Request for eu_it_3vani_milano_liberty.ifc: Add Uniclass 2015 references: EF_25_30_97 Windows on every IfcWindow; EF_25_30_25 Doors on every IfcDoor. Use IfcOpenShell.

First a look at what the model holds.

```python
import ifcopenshell

model = ifcopenshell.open("eu_it_3vani_milano_liberty.ifc")
print(model.schema)
print("classifications:", [c.Name for c in model.by_type("IfcClassification")])
for ifc_class in ("IfcDoor", "IfcRoof", "IfcStair", "IfcWall", "IfcWindow"):
    print(ifc_class, len(model.by_type(ifc_class)))
```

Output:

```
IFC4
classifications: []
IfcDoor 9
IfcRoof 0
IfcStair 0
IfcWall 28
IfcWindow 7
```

```python
import ifcopenshell
import ifcopenshell.api.classification

model = ifcopenshell.open("eu_it_3vani_milano_liberty.ifc")

system = ifcopenshell.api.classification.add_classification(model, classification="Uniclass 2015")

codes = {
    "IfcWindow": ("EF_25_30_97", "Windows"),
    "IfcDoor": ("EF_25_30_25", "Doors"),
}
for ifc_class, (code, name) in codes.items():
    products = model.by_type(ifc_class)
    ifcopenshell.api.classification.add_reference(
        model, products=products, classification=system, identification=code, name=name
    )
    print(code, len(products))

model.write("eu_it_3vani_milano_liberty_rev.ifc")
```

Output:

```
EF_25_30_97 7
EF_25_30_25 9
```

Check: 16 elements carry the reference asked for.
